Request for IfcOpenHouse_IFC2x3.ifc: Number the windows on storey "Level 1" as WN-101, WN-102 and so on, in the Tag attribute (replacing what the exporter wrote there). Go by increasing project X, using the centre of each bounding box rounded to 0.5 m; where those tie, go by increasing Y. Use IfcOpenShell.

First a look at what the model holds.

```python
import ifcopenshell
import ifcopenshell.util.element
import ifcopenshell.util.placement

model = ifcopenshell.open("IfcOpenHouse_IFC2x3.ifc")
print(model.schema)
storey = next(s for s in model.by_type("IfcBuildingStorey") if s.Name == "Level 1")
windows = [e for e in ifcopenshell.util.element.get_decomposition(storey) if e.is_a("IfcWindow")]
for e in sorted(windows, key=lambda e: e.id()):
    origin = ifcopenshell.util.placement.get_local_placement(e.ObjectPlacement)[:3, 3]
    print(e.id(), e.Tag, e.Name, origin.round(2) + 0.0, sep=" | ")
```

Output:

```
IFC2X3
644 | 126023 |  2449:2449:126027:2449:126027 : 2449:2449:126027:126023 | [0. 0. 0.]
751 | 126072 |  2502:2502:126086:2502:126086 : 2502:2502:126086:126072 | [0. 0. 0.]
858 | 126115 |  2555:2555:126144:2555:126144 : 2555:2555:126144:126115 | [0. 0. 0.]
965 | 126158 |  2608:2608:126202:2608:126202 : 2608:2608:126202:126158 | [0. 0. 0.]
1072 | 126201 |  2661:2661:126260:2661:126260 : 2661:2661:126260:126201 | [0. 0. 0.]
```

```python
import ifcopenshell
import ifcopenshell.geom
import ifcopenshell.util.element
import ifcopenshell.util.shape

model = ifcopenshell.open("IfcOpenHouse_IFC2x3.ifc")
settings = ifcopenshell.geom.settings()
settings.set("use-world-coords", True)


def centre(element):
    shape = ifcopenshell.geom.create_shape(settings, element)
    return ifcopenshell.util.shape.get_bbox_centroid(shape.geometry)


storey = next(s for s in model.by_type("IfcBuildingStorey") if s.Name == "Level 1")
windows = [e for e in ifcopenshell.util.element.get_decomposition(storey) if e.is_a("IfcWindow")]

# Insertion points can sit at a corner or the storey origin, so sort by the geometry (in metres).
centres = {e: centre(e) for e in windows}
windows.sort(key=lambda e: (round(centres[e][0] / 0.5), centres[e][1]))

for i, e in enumerate(windows, start=1):
    number = f"WN-1{i:02d}"
    e.Tag = number
    print(e.id(), number)

model.write("IfcOpenHouse_IFC2x3-out.ifc")
```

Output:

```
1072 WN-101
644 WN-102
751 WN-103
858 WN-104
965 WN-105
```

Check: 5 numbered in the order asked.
